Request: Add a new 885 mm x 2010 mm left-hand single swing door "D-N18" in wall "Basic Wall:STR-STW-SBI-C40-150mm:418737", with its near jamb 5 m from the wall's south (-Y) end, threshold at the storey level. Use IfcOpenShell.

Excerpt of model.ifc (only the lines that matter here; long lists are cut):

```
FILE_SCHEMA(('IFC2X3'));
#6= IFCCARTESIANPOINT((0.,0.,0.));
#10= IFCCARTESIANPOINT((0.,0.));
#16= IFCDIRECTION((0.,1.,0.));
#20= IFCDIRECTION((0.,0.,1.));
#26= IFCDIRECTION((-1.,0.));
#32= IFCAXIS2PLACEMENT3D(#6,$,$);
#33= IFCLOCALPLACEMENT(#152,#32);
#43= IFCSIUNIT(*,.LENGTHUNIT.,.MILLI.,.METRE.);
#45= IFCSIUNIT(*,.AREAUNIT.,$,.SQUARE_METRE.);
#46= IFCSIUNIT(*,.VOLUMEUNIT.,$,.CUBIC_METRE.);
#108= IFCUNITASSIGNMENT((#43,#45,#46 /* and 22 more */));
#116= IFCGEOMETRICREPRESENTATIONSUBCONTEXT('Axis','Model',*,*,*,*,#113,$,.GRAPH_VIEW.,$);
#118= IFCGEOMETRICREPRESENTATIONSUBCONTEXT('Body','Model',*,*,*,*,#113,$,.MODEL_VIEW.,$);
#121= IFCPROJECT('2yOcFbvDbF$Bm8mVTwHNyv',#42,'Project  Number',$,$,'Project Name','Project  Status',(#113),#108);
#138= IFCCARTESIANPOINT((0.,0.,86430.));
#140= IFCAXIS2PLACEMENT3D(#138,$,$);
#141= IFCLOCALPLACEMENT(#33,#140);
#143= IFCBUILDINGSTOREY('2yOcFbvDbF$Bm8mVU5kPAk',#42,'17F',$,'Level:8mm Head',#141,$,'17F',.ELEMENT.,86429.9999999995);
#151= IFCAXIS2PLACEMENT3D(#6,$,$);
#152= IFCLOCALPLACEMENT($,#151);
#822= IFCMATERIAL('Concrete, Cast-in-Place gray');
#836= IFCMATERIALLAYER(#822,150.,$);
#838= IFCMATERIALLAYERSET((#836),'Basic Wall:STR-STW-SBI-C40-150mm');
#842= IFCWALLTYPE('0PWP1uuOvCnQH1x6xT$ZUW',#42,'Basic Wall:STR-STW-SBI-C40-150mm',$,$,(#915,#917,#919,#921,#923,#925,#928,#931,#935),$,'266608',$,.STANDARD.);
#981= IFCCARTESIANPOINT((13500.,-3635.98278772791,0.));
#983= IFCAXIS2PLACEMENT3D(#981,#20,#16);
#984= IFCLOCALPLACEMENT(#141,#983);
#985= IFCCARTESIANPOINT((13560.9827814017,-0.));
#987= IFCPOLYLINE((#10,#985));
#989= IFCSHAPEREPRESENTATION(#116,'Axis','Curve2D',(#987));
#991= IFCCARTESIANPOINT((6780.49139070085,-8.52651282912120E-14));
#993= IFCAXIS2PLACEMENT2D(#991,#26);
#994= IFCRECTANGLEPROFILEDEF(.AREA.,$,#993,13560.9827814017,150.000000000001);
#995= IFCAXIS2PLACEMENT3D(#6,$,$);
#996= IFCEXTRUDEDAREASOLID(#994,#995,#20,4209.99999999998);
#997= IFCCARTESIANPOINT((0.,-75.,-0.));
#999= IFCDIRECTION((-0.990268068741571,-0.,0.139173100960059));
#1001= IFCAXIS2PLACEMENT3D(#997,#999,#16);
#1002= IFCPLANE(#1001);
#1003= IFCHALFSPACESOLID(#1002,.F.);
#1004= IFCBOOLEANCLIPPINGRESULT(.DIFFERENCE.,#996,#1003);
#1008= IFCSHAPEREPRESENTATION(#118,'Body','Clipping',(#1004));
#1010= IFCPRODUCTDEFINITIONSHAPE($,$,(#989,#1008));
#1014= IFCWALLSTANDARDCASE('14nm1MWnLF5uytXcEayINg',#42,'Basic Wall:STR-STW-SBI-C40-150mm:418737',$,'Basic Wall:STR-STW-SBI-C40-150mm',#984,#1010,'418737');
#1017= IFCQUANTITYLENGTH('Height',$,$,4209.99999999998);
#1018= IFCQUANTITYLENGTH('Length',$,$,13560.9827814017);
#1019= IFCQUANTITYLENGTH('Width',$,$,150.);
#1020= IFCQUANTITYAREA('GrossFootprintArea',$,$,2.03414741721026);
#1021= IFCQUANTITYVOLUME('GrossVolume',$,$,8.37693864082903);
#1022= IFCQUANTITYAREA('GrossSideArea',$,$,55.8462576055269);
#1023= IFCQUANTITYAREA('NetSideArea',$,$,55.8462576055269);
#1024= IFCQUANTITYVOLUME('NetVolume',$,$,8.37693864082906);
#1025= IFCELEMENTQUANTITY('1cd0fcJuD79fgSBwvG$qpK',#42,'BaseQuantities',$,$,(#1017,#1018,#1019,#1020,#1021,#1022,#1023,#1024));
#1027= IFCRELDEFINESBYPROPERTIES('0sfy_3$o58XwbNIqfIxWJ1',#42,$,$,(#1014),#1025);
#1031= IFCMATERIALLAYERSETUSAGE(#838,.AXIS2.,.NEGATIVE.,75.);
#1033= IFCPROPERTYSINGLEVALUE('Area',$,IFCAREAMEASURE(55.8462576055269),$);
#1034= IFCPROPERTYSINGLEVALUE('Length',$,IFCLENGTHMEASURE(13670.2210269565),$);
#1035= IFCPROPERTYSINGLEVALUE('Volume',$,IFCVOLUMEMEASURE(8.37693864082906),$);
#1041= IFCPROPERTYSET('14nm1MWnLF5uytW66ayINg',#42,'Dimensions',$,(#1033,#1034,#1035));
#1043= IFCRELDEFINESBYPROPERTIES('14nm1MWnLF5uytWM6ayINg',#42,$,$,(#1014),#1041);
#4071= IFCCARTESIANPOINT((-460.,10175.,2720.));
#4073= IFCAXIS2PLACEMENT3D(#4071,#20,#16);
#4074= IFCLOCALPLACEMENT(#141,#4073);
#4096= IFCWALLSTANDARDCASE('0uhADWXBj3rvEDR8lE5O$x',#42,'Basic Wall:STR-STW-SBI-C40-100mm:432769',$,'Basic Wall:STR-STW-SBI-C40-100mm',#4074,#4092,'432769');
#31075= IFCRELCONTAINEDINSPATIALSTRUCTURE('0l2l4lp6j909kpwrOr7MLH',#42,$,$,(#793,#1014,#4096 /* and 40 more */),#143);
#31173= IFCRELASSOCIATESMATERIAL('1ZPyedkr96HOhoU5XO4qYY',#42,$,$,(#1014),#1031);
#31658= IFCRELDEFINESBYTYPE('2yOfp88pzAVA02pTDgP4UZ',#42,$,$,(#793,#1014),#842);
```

```python
import numpy as np
import ifcopenshell
import ifcopenshell.api.feature
import ifcopenshell.api.geometry
import ifcopenshell.api.pset
import ifcopenshell.api.root
import ifcopenshell.api.spatial
import ifcopenshell.api.type
import ifcopenshell.geom
import ifcopenshell.util.element
import ifcopenshell.util.placement
import ifcopenshell.util.representation
import ifcopenshell.util.shape
import ifcopenshell.util.unit

model = ifcopenshell.open("model.ifc")
unit_scale = ifcopenshell.util.unit.calculate_unit_scale(model)
area_scale = ifcopenshell.util.unit.calculate_unit_scale(model, "AREAUNIT")
volume_scale = ifcopenshell.util.unit.calculate_unit_scale(model, "VOLUMEUNIT")
settings = ifcopenshell.geom.settings()


def volume(element):
    """Net volume in cubic metres, openings subtracted."""
    shape = ifcopenshell.geom.create_shape(settings, element)
    return ifcopenshell.util.shape.get_volume(shape.geometry)


wall = model.by_guid("14nm1MWnLF5uytXcEayINg")
storey = ifcopenshell.util.element.get_container(wall, ifc_class="IfcBuildingStorey")
context = ifcopenshell.util.representation.get_context(model, "Model", "Body", "MODEL_VIEW")
before = volume(wall)

width, height, from_end, sill = 0.885, 2.01, 5, 0.0  # metres

# The wall runs along its own X axis, and the end named is its -X end.
wall_shape = ifcopenshell.geom.create_shape(settings, wall)
x, y, z = ifcopenshell.util.shape.get_vertices(wall_shape.geometry).T
start = x.min() + from_end
face, thickness = float(y.min()), float(y.max() - y.min())
wall_matrix = ifcopenshell.util.placement.get_local_placement(wall.ObjectPlacement)
level = ifcopenshell.util.placement.get_local_placement(storey.ObjectPlacement)[2, 3]


def in_wall(x, y):
    """Placement at x, y metres in the wall's axes, at sill height."""
    matrix = wall_matrix.copy()
    matrix[:, 3] = wall_matrix @ np.array([x / unit_scale, y / unit_scale, 0.0, 1.0])
    matrix[2, 3] = level + sill / unit_scale
    return matrix


# Opening: a box that overshoots both wall faces by 50 mm.
opening = ifcopenshell.api.root.create_entity(model, ifc_class="IfcOpeningElement")
box = ifcopenshell.api.geometry.add_wall_representation(
    model, context=context, length=width, height=height, thickness=thickness + 0.1
)
ifcopenshell.api.geometry.assign_representation(model, product=opening, representation=box)
ifcopenshell.api.geometry.edit_object_placement(model, product=opening, matrix=in_wall(start, face - 0.05), is_si=False)
ifcopenshell.api.feature.add_feature(model, feature=opening, element=wall)

door = ifcopenshell.api.root.create_entity(model, ifc_class="IfcDoor", name="D-N18")
door.OverallWidth, door.OverallHeight = width / unit_scale, height / unit_scale
body = ifcopenshell.api.geometry.add_door_representation(
    model,
    context=context,
    overall_width=door.OverallWidth,
    overall_height=door.OverallHeight,
    operation_type="SINGLE_SWING_LEFT",
    lining_properties={"LiningDepth": thickness / unit_scale, "ThresholdDepth": thickness / unit_scale},
)
ifcopenshell.api.geometry.assign_representation(model, product=door, representation=body)
ifcopenshell.api.spatial.assign_container(model, products=[door], relating_structure=storey)
fills = ifcopenshell.api.feature.add_filling(model, opening=opening, element=door)
fills.OwnerHistory = door.OwnerHistory  # required in IFC2X3

# IFC2X3 keeps the operation on the door style.
style = ifcopenshell.api.root.create_entity(model, ifc_class="IfcDoorStyle", name="D-N18")
style.OperationType, style.ConstructionType = "SINGLE_SWING_LEFT", "NOTDEFINED"
style.ParameterTakesPrecedence = style.Sizeable = False
ifcopenshell.api.type.assign_type(model, related_objects=[door], relating_type=style)

# The lining spans the wall, so the door starts at the wall face.
ifcopenshell.api.geometry.edit_object_placement(model, product=door, matrix=in_wall(start, face), is_si=False)

after = volume(wall)

# Update the wall's stored quantities.
qto = model.by_id(ifcopenshell.util.element.get_pset(wall, "BaseQuantities", should_inherit=False)["id"])
ifcopenshell.api.pset.edit_qto(model, qto=qto, properties={
    "NetSideArea": after / thickness / area_scale,
    "NetVolume": after / volume_scale,
})
pset = model.by_id(ifcopenshell.util.element.get_pset(wall, "Dimensions", should_inherit=False)["id"])
ifcopenshell.api.pset.edit_pset(model, pset=pset, properties={
    "Area": model.create_entity("IfcAreaMeasure", after / thickness / area_scale),
    "Volume": model.create_entity("IfcVolumeMeasure", after / volume_scale),
})

print(f"wall volume {before:.3f} -> {after:.3f} m3")

model.write("model_v2.ifc")
```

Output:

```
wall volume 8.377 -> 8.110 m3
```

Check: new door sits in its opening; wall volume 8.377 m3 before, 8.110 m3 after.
